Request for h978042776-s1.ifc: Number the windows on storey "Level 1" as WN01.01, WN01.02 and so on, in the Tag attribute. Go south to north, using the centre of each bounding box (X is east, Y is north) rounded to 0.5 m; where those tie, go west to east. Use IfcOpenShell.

First a look at what the model holds.

```python
import ifcopenshell
import ifcopenshell.util.element
import ifcopenshell.util.placement

model = ifcopenshell.open("h978042776-s1.ifc")
print(model.schema)
storey = next(s for s in model.by_type("IfcBuildingStorey") if s.Name == "Level 1")
windows = [e for e in ifcopenshell.util.element.get_decomposition(storey) if e.is_a("IfcWindow")]
for e in sorted(windows, key=lambda e: e.id()):
    origin = ifcopenshell.util.placement.get_local_placement(e.ObjectPlacement)[:3, 3]
    print(e.id(), e.Tag, e.Name, origin.round(2) + 0.0, sep=" | ")
```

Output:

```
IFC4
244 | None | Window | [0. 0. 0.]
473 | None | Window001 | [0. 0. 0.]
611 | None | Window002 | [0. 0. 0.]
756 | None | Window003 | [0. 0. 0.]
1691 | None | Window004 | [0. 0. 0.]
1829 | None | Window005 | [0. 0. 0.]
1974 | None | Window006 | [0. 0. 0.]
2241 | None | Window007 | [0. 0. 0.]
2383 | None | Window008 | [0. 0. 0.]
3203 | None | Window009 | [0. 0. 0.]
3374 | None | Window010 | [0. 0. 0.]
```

```python
import ifcopenshell
import ifcopenshell.geom
import ifcopenshell.util.element
import ifcopenshell.util.shape

model = ifcopenshell.open("h978042776-s1.ifc")
settings = ifcopenshell.geom.settings()
settings.set("use-world-coords", True)


def centre(element):
    shape = ifcopenshell.geom.create_shape(settings, element)
    return ifcopenshell.util.shape.get_bbox_centroid(shape.geometry)


storey = next(s for s in model.by_type("IfcBuildingStorey") if s.Name == "Level 1")
windows = [e for e in ifcopenshell.util.element.get_decomposition(storey) if e.is_a("IfcWindow")]

# Insertion points can sit at a corner or the storey origin, so sort by the geometry (in metres).
centres = {e: centre(e) for e in windows}
windows.sort(key=lambda e: (round(centres[e][1] / 0.5), centres[e][0]))

for i, e in enumerate(windows, start=1):
    number = f"WN01.{i:02d}"
    e.Tag = number
    print(e.id(), number)

model.write("h978042776-s1_updated.ifc")
```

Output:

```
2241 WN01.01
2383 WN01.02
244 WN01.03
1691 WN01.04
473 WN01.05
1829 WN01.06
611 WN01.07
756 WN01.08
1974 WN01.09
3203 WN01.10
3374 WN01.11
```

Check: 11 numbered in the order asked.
